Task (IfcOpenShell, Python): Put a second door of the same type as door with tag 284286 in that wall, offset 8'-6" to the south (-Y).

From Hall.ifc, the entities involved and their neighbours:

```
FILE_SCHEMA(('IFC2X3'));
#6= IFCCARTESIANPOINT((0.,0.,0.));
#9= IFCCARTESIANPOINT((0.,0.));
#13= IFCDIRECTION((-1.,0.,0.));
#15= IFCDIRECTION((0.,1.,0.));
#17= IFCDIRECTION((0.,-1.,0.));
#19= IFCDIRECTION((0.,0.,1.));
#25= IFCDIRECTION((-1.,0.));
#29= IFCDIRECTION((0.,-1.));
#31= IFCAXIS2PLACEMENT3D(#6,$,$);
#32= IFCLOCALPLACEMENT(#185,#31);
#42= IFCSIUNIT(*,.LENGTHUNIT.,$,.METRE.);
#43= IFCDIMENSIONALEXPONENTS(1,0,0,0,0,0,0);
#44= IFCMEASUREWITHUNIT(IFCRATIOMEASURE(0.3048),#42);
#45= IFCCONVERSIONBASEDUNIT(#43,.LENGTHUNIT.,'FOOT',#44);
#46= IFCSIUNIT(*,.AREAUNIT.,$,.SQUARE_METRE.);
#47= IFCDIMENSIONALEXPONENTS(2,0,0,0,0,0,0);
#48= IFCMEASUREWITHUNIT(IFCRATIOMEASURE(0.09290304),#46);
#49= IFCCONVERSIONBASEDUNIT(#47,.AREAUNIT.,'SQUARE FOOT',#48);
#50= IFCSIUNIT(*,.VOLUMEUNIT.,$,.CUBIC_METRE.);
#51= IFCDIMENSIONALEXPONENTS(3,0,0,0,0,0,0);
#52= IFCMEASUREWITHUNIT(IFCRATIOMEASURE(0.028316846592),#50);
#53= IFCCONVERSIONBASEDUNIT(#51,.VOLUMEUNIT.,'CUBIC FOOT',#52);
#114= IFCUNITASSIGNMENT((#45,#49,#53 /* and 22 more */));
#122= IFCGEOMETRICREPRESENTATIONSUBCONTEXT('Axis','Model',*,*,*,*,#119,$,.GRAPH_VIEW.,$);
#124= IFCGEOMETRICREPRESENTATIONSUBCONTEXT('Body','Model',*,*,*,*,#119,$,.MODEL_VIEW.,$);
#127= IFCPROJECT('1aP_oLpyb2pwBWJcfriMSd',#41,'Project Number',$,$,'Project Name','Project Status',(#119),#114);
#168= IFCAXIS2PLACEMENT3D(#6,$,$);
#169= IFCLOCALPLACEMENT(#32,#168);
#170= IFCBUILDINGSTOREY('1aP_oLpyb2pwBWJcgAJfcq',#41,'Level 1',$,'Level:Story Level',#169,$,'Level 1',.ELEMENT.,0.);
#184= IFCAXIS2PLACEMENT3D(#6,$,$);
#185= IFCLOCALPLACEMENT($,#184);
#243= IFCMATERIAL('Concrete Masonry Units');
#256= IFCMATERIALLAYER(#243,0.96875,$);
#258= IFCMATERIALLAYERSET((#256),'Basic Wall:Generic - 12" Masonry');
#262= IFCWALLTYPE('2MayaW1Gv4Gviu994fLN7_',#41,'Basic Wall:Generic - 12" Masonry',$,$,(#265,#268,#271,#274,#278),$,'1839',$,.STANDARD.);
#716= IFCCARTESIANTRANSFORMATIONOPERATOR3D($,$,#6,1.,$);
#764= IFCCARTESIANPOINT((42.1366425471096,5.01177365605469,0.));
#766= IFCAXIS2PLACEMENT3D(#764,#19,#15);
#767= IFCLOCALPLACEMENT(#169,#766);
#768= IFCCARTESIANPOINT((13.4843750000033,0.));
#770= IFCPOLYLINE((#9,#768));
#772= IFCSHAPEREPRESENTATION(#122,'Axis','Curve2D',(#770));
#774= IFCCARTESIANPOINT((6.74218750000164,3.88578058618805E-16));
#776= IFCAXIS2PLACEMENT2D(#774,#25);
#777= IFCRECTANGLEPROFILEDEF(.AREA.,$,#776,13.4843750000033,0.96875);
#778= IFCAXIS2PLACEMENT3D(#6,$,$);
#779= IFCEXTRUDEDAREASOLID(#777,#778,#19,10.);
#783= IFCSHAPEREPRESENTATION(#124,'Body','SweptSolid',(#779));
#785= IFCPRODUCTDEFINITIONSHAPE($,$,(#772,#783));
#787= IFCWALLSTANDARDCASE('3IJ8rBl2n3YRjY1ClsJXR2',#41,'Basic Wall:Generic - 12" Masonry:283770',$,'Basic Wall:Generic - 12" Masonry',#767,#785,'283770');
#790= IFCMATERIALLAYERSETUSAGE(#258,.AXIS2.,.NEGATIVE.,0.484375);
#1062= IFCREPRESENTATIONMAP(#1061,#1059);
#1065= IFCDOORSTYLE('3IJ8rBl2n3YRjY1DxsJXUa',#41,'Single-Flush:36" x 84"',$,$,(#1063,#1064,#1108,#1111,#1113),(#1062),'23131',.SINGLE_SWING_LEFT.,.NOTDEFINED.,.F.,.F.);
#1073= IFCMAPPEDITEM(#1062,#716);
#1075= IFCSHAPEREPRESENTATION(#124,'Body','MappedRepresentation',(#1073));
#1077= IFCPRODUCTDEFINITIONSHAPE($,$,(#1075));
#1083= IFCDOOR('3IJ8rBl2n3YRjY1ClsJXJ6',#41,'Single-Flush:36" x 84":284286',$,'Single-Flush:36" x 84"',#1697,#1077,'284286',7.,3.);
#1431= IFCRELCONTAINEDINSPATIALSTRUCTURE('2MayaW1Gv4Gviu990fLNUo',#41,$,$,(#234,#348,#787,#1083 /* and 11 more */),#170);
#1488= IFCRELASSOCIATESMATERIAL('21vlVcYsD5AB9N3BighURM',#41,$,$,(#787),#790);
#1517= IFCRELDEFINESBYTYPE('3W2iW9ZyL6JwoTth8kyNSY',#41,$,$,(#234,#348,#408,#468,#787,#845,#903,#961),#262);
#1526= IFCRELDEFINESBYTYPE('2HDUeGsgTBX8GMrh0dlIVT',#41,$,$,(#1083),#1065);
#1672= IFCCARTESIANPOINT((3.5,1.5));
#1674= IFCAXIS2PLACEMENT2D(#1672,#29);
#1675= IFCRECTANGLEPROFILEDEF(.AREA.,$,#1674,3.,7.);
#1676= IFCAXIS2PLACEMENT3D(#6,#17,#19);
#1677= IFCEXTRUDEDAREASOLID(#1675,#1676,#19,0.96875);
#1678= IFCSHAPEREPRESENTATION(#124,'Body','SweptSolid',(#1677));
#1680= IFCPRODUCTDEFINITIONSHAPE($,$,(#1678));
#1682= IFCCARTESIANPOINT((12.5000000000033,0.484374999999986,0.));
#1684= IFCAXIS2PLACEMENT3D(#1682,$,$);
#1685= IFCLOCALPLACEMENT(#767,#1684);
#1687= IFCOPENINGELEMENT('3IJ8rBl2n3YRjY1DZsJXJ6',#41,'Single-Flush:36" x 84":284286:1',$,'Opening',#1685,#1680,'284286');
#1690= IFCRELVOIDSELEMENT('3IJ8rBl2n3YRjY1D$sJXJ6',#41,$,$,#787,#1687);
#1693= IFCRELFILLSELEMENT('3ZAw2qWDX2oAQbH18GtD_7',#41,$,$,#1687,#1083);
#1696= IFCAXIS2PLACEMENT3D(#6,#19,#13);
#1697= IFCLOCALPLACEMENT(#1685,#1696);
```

```python
import ifcopenshell
import ifcopenshell.api.feature
import ifcopenshell.api.geometry
import ifcopenshell.api.root
import ifcopenshell.geom
import ifcopenshell.util.element
import ifcopenshell.util.placement
import ifcopenshell.util.shape
import ifcopenshell.util.unit

model = ifcopenshell.open("Hall.ifc")
unit_scale = ifcopenshell.util.unit.calculate_unit_scale(model)
settings = ifcopenshell.geom.settings()


def volume(element):
    """Net volume in cubic metres, openings subtracted."""
    shape = ifcopenshell.geom.create_shape(settings, element)
    return ifcopenshell.util.shape.get_volume(shape.geometry)


def reuse_history(source, copy):
    """copy_class also copies each property set's owner history, people and application; keep the originals."""
    for rel in copy.IsDefinedBy:
        if rel.is_a("IfcRelDefinesByProperties") and (history := rel.RelatingPropertyDefinition.OwnerHistory):
            rel.RelatingPropertyDefinition.OwnerHistory = source.OwnerHistory
            ifcopenshell.util.element.remove_deep2(model, history)


door = model.by_guid("3IJ8rBl2n3YRjY1ClsJXJ6")
opening = door.FillsVoids[0].RelatingOpeningElement
wall = opening.VoidsElements[0].RelatingBuildingElement
before = volume(wall)
shift = ifcopenshell.util.placement.get_local_placement(wall.ObjectPlacement)[:3, 0] * -102 * 0.0254 / unit_scale

# copy_class copies the void relationship, type, container and properties, but no geometry.
new_opening = ifcopenshell.api.root.copy_class(model, product=opening)
new_opening.Representation = ifcopenshell.util.element.copy_deep(
    model, opening.Representation, exclude=["IfcGeometricRepresentationContext", "IfcRepresentationMap"]
)
new_opening.Name = 'Single-Flush:36" x 84"'
new_opening.Tag = None
new_door = ifcopenshell.api.root.copy_class(model, product=door)
new_door.Representation = ifcopenshell.util.element.copy_deep(
    model, door.Representation, exclude=["IfcGeometricRepresentationContext", "IfcRepresentationMap"]
)
new_door.Name = 'Single-Flush:36" x 84"'
new_door.Tag = None
reuse_history(door, new_door)
fills = ifcopenshell.api.feature.add_filling(model, opening=new_opening, element=new_door)
fills.OwnerHistory = new_door.OwnerHistory  # required in IFC2X3

for old, new in ((opening, new_opening), (door, new_door)):
    matrix = ifcopenshell.util.placement.get_local_placement(old.ObjectPlacement)
    matrix[:3, 3] += shift
    ifcopenshell.api.geometry.edit_object_placement(model, product=new, matrix=matrix, is_si=False)

after = volume(wall)

print(f"wall volume {before:.3f} -> {after:.3f} m3")

model.write("Hall_v2.ifc")
```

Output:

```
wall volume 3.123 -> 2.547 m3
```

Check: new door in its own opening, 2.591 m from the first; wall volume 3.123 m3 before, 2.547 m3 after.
